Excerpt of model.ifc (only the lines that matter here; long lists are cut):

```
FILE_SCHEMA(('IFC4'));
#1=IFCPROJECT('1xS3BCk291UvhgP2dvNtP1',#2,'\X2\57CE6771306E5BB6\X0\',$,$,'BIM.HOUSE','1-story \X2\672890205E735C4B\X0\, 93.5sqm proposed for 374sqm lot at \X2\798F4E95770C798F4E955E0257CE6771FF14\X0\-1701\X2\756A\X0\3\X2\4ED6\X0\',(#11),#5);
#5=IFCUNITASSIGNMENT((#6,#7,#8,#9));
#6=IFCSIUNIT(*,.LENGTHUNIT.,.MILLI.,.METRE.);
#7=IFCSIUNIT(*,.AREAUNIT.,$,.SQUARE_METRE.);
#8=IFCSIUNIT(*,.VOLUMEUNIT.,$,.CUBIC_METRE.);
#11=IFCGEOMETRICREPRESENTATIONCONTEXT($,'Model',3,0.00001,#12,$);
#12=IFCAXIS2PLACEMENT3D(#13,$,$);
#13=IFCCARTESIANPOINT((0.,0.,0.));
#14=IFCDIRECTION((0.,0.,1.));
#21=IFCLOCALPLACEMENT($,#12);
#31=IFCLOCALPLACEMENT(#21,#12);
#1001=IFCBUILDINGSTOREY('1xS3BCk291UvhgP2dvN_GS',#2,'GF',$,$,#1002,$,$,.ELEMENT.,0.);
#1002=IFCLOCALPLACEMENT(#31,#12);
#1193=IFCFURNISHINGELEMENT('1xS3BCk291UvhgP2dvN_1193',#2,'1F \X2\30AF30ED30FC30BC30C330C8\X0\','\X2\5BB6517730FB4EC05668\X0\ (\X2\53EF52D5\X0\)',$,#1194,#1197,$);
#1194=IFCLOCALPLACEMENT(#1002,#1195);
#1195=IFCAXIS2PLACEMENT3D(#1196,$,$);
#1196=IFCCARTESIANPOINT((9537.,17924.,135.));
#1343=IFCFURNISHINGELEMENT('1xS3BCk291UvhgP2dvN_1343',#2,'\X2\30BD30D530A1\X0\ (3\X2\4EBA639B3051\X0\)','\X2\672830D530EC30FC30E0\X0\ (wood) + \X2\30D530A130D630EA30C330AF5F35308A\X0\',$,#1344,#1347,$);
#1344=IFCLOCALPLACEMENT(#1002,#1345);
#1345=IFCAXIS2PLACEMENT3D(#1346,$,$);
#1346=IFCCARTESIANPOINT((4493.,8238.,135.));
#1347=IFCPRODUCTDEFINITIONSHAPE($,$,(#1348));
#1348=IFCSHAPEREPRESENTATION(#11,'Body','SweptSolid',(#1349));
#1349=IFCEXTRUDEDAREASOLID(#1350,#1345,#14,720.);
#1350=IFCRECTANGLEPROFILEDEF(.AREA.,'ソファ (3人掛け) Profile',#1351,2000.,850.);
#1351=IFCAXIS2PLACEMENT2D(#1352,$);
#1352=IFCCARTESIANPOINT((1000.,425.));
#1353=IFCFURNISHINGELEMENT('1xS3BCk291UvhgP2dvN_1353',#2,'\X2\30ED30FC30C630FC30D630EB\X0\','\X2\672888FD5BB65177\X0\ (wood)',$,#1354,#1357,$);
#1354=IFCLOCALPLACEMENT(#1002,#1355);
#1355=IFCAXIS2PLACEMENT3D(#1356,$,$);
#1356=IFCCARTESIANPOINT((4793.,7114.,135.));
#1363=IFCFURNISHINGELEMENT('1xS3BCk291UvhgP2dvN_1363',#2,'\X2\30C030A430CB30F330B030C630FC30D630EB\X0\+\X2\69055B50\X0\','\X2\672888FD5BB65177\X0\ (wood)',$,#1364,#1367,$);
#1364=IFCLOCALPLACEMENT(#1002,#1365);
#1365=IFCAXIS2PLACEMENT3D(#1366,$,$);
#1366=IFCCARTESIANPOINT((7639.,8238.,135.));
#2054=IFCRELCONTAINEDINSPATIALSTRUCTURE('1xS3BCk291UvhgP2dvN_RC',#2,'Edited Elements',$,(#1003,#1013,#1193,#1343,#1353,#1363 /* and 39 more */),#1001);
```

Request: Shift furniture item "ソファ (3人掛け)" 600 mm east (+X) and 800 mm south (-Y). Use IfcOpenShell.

```python
import ifcopenshell
import ifcopenshell.api.geometry
import ifcopenshell.util.placement

model = ifcopenshell.open("model.ifc")

item = model.by_id(1343)
matrix = ifcopenshell.util.placement.get_local_placement(item.ObjectPlacement)
matrix[0, 3] += 600.0
matrix[1, 3] -= 800.0
ifcopenshell.api.geometry.edit_object_placement(model, product=item, matrix=matrix, is_si=False)

print(ifcopenshell.util.placement.get_local_placement(item.ObjectPlacement).round(3) + 0.0)

model.write("model_v2.ifc")
```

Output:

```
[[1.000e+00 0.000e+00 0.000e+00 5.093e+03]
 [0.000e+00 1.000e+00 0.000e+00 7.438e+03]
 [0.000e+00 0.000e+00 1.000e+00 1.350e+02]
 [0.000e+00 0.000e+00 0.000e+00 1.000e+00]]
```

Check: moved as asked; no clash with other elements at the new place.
